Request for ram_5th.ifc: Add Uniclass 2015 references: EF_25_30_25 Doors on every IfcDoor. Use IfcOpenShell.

First a look at what the model holds.

```python
import ifcopenshell

model = ifcopenshell.open("ram_5th.ifc")
print(model.schema)
print("classifications:", [c.Name for c in model.by_type("IfcClassification")])
for ifc_class in ("IfcDoor", "IfcRoof", "IfcStair", "IfcWall", "IfcWindow"):
    print(ifc_class, len(model.by_type(ifc_class)))
```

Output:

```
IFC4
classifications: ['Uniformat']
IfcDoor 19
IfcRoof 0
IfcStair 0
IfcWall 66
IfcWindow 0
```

```python
import ifcopenshell
import ifcopenshell.api.classification

model = ifcopenshell.open("ram_5th.ifc")

system = ifcopenshell.api.classification.add_classification(model, classification="Uniclass 2015")

codes = {
    "IfcDoor": ("EF_25_30_25", "Doors"),
}
for ifc_class, (code, name) in codes.items():
    products = model.by_type(ifc_class)
    ifcopenshell.api.classification.add_reference(
        model, products=products, classification=system, identification=code, name=name
    )
    print(code, len(products))

model.write("ram_5th_edited.ifc")
```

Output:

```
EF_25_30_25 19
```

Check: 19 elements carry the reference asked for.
